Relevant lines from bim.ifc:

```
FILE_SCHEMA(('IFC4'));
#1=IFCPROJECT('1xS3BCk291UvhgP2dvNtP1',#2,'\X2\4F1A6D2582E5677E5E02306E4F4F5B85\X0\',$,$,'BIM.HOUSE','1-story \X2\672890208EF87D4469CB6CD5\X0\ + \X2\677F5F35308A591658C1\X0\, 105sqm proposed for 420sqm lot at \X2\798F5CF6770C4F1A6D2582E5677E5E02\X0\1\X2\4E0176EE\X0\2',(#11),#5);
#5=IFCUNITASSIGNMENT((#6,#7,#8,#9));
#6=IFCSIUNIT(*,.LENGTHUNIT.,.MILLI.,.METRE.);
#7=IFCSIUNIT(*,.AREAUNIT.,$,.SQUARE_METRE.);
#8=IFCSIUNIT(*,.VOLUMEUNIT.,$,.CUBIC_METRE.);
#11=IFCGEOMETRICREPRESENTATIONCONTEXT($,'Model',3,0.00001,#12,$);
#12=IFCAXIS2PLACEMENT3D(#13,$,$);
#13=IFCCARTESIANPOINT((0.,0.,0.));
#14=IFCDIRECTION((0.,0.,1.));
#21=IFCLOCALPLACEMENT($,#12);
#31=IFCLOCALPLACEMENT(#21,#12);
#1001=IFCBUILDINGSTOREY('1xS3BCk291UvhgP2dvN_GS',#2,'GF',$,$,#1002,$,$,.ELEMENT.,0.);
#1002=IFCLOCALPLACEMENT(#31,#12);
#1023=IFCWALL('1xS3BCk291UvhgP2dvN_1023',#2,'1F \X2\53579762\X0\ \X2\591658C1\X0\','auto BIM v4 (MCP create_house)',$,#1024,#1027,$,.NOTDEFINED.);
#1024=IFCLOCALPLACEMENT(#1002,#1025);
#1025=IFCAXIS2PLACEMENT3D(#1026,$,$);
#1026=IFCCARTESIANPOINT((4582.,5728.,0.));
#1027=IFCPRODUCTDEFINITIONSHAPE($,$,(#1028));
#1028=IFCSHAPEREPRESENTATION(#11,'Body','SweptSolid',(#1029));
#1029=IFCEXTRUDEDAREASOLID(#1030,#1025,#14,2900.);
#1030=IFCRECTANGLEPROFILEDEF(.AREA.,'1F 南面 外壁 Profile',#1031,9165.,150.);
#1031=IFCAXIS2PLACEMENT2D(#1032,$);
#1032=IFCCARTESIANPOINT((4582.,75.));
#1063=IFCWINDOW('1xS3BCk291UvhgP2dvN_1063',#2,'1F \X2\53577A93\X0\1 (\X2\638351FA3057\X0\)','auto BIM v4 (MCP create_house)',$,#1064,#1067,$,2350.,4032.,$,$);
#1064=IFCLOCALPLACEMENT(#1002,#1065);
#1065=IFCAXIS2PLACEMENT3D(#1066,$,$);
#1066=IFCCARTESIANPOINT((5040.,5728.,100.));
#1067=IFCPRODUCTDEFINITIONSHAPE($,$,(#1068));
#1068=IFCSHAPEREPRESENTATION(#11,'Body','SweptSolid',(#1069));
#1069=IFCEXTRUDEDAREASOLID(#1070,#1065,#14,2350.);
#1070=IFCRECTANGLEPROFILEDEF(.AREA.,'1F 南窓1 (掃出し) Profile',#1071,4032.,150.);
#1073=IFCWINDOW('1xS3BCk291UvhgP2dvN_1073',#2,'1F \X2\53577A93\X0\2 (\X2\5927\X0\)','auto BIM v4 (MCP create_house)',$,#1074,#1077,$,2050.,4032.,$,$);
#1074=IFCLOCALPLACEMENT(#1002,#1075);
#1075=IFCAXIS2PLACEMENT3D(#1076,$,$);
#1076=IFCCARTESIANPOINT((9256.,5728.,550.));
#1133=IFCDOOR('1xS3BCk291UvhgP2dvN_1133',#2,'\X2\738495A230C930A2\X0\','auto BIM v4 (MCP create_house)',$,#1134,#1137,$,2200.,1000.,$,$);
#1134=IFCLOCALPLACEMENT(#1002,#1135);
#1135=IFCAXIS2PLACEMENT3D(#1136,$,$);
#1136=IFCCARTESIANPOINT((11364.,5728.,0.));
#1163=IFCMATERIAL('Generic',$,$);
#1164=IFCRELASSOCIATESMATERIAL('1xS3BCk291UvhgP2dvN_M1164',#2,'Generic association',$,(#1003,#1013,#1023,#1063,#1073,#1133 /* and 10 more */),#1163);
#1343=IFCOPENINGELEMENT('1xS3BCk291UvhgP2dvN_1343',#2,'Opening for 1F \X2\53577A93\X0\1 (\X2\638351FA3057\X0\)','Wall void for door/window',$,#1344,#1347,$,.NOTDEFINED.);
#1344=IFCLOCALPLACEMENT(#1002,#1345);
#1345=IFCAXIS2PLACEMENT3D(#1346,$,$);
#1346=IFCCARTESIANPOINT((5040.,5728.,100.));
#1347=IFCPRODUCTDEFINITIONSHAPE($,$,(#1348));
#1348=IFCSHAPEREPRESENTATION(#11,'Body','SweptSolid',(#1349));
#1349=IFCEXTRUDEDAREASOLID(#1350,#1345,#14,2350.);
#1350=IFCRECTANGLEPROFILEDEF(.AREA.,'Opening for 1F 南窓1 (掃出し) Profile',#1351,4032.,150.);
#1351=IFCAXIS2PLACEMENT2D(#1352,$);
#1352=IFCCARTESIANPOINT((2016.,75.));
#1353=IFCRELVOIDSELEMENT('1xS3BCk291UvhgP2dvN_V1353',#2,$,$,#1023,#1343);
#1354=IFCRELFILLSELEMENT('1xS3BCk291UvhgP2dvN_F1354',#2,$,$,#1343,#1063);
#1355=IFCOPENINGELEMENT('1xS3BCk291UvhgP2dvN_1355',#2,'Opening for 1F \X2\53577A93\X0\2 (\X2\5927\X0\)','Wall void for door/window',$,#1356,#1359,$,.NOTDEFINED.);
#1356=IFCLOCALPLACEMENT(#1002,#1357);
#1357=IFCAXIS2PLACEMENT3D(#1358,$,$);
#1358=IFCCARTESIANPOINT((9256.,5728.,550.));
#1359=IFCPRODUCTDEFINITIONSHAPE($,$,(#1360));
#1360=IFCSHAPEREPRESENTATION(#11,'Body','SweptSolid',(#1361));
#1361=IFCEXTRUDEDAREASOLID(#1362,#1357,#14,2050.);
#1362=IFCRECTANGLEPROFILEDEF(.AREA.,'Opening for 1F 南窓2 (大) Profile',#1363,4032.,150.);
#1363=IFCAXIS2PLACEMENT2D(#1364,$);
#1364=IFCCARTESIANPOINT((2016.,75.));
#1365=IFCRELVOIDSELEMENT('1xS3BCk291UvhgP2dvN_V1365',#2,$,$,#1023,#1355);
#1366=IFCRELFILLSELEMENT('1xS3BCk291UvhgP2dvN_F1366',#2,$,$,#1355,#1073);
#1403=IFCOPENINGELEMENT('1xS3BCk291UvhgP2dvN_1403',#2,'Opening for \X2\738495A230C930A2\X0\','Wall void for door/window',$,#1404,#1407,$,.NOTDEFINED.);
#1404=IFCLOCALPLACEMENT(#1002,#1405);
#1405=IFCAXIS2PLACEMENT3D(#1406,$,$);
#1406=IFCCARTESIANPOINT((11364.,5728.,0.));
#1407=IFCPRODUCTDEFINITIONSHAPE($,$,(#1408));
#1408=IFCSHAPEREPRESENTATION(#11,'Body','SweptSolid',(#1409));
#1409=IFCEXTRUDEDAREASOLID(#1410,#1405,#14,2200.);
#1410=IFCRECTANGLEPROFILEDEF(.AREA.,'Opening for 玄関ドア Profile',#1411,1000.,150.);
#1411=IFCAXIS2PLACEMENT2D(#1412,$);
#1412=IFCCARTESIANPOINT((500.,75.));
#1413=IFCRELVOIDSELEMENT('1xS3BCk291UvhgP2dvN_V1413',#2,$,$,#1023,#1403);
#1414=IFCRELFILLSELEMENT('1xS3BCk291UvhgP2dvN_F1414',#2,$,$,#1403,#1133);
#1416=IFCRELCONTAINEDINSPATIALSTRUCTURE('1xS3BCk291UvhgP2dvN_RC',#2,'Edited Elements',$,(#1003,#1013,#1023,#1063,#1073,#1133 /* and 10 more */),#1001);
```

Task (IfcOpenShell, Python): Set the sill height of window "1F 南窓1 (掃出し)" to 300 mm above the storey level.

```python
import numpy as np
import ifcopenshell
import ifcopenshell.api.geometry
import ifcopenshell.geom
import ifcopenshell.util.element
import ifcopenshell.util.placement
import ifcopenshell.util.shape
import ifcopenshell.util.unit

model = ifcopenshell.open("bim.ifc")
unit_scale = ifcopenshell.util.unit.calculate_unit_scale(model)

window = model.by_guid("1xS3BCk291UvhgP2dvN_1063")
opening = window.FillsVoids[0].RelatingOpeningElement
storey = ifcopenshell.util.element.get_container(window, ifc_class="IfcBuildingStorey")
level = ifcopenshell.util.placement.get_local_placement(storey.ObjectPlacement)[2, 3]

# The opening's origin need not be at the sill, so measure its lowest point.
shape = ifcopenshell.geom.create_shape(ifcopenshell.geom.settings(), opening)
bottom = ifcopenshell.util.shape.get_shape_bottom_elevation(shape, shape.geometry) / unit_scale
dz = level + 0.3 / unit_scale - bottom

shift = np.array([0.0, 0.0, dz])
# The window is not placed relative to its opening, so move both.
for product in (opening, window):
    matrix = ifcopenshell.util.placement.get_local_placement(product.ObjectPlacement)
    matrix[:3, 3] += shift
    ifcopenshell.api.geometry.edit_object_placement(model, product=product, matrix=matrix, is_si=False)

print(f"moved by {dz * unit_scale:+.3f} m")

model.write("bim_updated.ifc")
```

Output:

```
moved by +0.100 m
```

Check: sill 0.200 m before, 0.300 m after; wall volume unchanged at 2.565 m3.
